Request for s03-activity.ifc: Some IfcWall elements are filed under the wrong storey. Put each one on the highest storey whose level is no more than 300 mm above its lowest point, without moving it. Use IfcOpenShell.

First a look at what the model holds.

```python
import ifcopenshell
import ifcopenshell.util.element
import ifcopenshell.util.placement

model = ifcopenshell.open("s03-activity.ifc")
print(model.schema)
for storey in model.by_type("IfcBuildingStorey"):
    level = ifcopenshell.util.placement.get_storey_elevation(storey)
    count = sum(e.is_a("IfcWall") for e in ifcopenshell.util.element.get_contained(storey))
    print(storey.id(), storey.Name, round(level, 3), count, sep=" | ")
```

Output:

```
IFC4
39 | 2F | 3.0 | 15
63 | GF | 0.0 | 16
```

```python
import ifcopenshell
import ifcopenshell.api.spatial
import ifcopenshell.geom
import ifcopenshell.util.element
import ifcopenshell.util.placement
import ifcopenshell.util.shape
import ifcopenshell.util.unit

model = ifcopenshell.open("s03-activity.ifc")
unit_scale = ifcopenshell.util.unit.calculate_unit_scale(model)
settings = ifcopenshell.geom.settings()

levels = sorted(
    ((ifcopenshell.util.placement.get_storey_elevation(s) * unit_scale, s) for s in model.by_type("IfcBuildingStorey")),
    key=lambda pair: pair[0],
)

for e in model.by_type("IfcWall"):
    current = e.ContainedInStructure[0].RelatingStructure if e.ContainedInStructure else None
    if current is None or not current.is_a("IfcBuildingStorey"):
        continue
    shape = ifcopenshell.geom.create_shape(settings, e)
    bottom = ifcopenshell.util.shape.get_shape_bottom_elevation(shape, shape.geometry)
    below = [s for level, s in levels if level <= bottom + 0.3]
    storey = below[-1] if below else levels[0][1]
    if storey != current:
        # assign_container keeps the world position.
        ifcopenshell.api.spatial.assign_container(model, products=[e], relating_structure=storey)
        print(e.id(), current.Name, "->", storey.Name)

model.write("s03-activity_updated.ifc")
```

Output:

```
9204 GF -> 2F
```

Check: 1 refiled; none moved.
